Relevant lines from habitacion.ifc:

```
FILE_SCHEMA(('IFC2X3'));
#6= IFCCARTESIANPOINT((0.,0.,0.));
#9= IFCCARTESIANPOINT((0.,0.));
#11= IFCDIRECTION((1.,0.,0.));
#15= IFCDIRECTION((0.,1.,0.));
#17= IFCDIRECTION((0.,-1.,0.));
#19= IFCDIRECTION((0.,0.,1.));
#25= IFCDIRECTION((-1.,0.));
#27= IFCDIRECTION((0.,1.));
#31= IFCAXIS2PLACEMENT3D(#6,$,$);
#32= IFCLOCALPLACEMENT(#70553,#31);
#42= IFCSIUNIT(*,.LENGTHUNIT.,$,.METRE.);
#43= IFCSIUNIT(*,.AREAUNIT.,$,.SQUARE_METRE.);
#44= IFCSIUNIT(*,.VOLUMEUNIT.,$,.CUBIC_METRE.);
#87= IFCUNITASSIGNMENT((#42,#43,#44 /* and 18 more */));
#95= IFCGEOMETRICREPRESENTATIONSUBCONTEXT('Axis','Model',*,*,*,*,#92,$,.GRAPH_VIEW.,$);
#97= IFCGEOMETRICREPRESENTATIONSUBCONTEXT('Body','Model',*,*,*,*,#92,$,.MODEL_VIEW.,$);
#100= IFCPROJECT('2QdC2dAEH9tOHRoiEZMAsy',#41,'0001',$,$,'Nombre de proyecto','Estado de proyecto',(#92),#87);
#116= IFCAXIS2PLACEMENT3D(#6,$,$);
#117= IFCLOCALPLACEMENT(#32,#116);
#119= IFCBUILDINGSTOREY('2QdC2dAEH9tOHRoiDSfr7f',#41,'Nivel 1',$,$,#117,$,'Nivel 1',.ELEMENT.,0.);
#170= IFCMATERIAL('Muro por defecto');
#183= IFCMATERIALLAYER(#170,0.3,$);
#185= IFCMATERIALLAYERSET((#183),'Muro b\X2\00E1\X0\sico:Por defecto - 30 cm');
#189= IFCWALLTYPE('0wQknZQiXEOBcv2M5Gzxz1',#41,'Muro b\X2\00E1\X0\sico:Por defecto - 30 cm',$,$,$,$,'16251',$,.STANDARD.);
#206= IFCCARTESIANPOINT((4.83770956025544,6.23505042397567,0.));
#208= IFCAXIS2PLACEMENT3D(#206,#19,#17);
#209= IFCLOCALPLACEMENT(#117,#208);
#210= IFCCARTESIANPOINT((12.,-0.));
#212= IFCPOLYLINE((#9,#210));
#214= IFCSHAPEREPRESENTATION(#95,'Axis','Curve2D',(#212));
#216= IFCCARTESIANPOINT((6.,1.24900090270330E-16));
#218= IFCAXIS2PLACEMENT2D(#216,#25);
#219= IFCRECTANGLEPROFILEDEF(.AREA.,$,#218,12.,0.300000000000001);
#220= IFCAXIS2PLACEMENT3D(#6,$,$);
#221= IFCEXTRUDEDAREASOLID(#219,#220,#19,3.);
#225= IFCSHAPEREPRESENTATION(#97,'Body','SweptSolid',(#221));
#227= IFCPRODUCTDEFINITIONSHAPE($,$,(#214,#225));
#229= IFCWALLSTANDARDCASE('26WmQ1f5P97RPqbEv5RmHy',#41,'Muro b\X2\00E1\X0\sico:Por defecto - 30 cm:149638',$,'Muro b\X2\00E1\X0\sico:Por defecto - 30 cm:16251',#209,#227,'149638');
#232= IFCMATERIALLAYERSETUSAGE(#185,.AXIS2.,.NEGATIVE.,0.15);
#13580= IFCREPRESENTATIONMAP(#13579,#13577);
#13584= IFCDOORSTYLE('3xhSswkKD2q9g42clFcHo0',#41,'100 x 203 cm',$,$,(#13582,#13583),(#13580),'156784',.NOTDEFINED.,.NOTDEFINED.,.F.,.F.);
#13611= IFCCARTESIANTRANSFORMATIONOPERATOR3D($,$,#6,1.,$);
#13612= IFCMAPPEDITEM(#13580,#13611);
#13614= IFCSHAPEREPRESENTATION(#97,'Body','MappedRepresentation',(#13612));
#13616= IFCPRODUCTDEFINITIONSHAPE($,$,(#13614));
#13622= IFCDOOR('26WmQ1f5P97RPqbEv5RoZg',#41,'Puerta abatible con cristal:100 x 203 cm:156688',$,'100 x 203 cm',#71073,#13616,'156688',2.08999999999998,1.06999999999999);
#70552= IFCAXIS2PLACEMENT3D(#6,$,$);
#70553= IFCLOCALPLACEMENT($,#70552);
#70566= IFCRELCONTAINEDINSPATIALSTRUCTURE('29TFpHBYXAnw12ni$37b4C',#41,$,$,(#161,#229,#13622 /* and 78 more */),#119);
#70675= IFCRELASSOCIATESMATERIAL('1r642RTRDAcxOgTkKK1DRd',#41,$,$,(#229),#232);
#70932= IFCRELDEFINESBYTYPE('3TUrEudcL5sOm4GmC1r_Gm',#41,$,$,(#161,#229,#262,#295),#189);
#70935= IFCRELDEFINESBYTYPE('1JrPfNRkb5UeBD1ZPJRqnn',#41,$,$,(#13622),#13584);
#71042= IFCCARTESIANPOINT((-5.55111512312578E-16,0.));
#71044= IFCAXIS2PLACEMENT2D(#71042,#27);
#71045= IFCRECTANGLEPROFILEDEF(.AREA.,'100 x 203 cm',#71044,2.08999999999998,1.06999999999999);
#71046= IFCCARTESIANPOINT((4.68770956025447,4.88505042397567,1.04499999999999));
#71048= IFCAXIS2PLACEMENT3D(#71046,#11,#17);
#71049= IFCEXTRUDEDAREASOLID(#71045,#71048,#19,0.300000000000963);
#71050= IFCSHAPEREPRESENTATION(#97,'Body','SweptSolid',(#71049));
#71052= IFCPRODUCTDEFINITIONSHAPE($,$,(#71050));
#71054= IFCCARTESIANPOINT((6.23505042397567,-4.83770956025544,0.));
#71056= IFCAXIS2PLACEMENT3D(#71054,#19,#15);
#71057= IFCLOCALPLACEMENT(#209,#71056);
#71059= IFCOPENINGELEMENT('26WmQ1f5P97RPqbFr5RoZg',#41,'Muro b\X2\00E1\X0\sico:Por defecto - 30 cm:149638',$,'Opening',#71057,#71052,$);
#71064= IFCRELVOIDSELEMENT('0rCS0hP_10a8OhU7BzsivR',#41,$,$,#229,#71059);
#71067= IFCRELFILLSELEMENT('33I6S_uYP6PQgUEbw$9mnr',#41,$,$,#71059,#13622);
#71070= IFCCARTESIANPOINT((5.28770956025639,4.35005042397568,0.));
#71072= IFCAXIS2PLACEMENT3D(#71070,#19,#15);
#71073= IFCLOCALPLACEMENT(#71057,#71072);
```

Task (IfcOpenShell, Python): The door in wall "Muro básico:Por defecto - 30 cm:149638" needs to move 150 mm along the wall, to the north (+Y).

```python
import ifcopenshell
import ifcopenshell.api.geometry
import ifcopenshell.util.placement
import ifcopenshell.util.unit

model = ifcopenshell.open("habitacion.ifc")
unit_scale = ifcopenshell.util.unit.calculate_unit_scale(model)

door = model.by_guid("26WmQ1f5P97RPqbEv5RoZg")
opening = door.FillsVoids[0].RelatingOpeningElement
wall = opening.VoidsElements[0].RelatingBuildingElement

wall_matrix = ifcopenshell.util.placement.get_local_placement(wall.ObjectPlacement)
shift = wall_matrix[:3, 0] * -0.15 / unit_scale
before = ifcopenshell.util.placement.get_local_placement(door.ObjectPlacement)[:3, 3].copy()

# The door is placed relative to its opening, so it follows when the opening moves.
matrix = ifcopenshell.util.placement.get_local_placement(opening.ObjectPlacement)
matrix[:3, 3] += shift
ifcopenshell.api.geometry.edit_object_placement(
    model, product=opening, matrix=matrix, is_si=False, should_transform_children=True
)

after = ifcopenshell.util.placement.get_local_placement(door.ObjectPlacement)[:3, 3]
print("door moved by", (after - before).round(3) + 0.0)

model.write("habitacion_rev.ifc")
```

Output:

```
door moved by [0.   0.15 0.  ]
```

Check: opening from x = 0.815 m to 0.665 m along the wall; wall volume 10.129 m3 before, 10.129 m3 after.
